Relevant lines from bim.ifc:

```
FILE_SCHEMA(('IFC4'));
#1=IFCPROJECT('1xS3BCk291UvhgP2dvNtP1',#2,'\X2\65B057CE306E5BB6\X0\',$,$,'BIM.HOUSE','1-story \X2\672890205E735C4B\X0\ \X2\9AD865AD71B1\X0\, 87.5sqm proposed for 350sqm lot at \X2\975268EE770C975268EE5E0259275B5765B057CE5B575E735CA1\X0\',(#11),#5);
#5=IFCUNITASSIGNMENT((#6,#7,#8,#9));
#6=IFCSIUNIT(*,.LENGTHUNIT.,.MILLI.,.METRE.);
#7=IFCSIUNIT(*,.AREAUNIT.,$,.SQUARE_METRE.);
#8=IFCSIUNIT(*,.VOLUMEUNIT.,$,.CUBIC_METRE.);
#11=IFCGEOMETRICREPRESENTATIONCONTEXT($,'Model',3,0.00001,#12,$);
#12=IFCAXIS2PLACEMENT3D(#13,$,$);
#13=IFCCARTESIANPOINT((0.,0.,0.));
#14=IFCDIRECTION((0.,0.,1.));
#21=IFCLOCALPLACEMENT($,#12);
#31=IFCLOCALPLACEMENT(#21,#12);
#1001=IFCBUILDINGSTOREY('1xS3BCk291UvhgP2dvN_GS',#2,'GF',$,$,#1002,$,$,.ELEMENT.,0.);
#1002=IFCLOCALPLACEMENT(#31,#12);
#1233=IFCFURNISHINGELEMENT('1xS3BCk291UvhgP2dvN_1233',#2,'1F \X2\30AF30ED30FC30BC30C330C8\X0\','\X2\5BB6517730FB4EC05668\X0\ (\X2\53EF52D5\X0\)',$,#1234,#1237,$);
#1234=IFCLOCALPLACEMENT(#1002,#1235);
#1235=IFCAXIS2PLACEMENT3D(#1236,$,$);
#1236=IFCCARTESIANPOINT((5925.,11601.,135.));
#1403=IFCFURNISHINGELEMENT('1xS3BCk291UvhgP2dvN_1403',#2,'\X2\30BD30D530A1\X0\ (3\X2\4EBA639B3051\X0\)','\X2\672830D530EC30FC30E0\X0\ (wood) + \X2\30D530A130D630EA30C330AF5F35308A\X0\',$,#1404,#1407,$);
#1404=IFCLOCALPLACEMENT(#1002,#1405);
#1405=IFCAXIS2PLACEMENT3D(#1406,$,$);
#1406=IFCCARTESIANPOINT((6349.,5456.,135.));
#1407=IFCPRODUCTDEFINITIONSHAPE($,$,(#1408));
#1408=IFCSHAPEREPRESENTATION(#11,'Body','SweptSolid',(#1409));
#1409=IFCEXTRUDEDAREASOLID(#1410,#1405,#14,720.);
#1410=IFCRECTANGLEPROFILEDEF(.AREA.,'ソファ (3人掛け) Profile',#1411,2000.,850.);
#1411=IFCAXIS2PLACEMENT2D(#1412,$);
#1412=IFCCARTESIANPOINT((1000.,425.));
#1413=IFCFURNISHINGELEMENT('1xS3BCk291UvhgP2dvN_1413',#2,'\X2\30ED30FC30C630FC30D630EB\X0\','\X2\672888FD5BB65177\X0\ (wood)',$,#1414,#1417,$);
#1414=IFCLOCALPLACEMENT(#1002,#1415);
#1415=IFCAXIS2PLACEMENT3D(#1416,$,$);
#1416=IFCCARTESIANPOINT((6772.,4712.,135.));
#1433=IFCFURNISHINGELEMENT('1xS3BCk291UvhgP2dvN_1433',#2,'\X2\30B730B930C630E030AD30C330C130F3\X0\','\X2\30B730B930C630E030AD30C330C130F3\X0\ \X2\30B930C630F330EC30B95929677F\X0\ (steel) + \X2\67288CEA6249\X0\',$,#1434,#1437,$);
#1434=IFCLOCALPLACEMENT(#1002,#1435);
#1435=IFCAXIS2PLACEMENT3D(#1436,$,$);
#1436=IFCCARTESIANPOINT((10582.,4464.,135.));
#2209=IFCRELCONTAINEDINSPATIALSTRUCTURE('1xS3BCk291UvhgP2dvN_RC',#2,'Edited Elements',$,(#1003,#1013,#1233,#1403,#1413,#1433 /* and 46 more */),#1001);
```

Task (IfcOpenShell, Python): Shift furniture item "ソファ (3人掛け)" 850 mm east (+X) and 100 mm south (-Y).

```python
import ifcopenshell
import ifcopenshell.api.geometry
import ifcopenshell.util.placement

model = ifcopenshell.open("bim.ifc")

item = model.by_guid("1xS3BCk291UvhgP2dvN_1403")
matrix = ifcopenshell.util.placement.get_local_placement(item.ObjectPlacement)
matrix[0, 3] += 850.0
matrix[1, 3] -= 100.0
ifcopenshell.api.geometry.edit_object_placement(model, product=item, matrix=matrix, is_si=False)

print(ifcopenshell.util.placement.get_local_placement(item.ObjectPlacement).round(3) + 0.0)

model.write("bim_updated.ifc")
```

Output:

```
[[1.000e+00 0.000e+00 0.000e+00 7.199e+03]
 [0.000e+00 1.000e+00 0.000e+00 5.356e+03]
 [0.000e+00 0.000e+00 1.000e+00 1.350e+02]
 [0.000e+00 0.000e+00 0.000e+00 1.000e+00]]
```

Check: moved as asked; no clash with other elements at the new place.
